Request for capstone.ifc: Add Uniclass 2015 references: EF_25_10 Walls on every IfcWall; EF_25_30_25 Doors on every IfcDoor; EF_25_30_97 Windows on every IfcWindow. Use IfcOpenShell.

First a look at what the model holds.

```python
import ifcopenshell

model = ifcopenshell.open("capstone.ifc")
print(model.schema)
print("classifications:", [c.Name for c in model.by_type("IfcClassification")])
for ifc_class in ("IfcDoor", "IfcRoof", "IfcStair", "IfcWall", "IfcWindow"):
    print(ifc_class, len(model.by_type(ifc_class)))
```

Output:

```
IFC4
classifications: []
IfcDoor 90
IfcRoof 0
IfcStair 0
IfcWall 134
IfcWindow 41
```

```python
import ifcopenshell
import ifcopenshell.api.classification

model = ifcopenshell.open("capstone.ifc")

system = ifcopenshell.api.classification.add_classification(model, classification="Uniclass 2015")

codes = {
    "IfcWall": ("EF_25_10", "Walls"),
    "IfcDoor": ("EF_25_30_25", "Doors"),
    "IfcWindow": ("EF_25_30_97", "Windows"),
}
for ifc_class, (code, name) in codes.items():
    products = model.by_type(ifc_class)
    ifcopenshell.api.classification.add_reference(
        model, products=products, classification=system, identification=code, name=name
    )
    print(code, len(products))

model.write("capstone_edited.ifc")
```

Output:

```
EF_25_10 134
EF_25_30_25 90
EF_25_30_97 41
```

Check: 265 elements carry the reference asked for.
